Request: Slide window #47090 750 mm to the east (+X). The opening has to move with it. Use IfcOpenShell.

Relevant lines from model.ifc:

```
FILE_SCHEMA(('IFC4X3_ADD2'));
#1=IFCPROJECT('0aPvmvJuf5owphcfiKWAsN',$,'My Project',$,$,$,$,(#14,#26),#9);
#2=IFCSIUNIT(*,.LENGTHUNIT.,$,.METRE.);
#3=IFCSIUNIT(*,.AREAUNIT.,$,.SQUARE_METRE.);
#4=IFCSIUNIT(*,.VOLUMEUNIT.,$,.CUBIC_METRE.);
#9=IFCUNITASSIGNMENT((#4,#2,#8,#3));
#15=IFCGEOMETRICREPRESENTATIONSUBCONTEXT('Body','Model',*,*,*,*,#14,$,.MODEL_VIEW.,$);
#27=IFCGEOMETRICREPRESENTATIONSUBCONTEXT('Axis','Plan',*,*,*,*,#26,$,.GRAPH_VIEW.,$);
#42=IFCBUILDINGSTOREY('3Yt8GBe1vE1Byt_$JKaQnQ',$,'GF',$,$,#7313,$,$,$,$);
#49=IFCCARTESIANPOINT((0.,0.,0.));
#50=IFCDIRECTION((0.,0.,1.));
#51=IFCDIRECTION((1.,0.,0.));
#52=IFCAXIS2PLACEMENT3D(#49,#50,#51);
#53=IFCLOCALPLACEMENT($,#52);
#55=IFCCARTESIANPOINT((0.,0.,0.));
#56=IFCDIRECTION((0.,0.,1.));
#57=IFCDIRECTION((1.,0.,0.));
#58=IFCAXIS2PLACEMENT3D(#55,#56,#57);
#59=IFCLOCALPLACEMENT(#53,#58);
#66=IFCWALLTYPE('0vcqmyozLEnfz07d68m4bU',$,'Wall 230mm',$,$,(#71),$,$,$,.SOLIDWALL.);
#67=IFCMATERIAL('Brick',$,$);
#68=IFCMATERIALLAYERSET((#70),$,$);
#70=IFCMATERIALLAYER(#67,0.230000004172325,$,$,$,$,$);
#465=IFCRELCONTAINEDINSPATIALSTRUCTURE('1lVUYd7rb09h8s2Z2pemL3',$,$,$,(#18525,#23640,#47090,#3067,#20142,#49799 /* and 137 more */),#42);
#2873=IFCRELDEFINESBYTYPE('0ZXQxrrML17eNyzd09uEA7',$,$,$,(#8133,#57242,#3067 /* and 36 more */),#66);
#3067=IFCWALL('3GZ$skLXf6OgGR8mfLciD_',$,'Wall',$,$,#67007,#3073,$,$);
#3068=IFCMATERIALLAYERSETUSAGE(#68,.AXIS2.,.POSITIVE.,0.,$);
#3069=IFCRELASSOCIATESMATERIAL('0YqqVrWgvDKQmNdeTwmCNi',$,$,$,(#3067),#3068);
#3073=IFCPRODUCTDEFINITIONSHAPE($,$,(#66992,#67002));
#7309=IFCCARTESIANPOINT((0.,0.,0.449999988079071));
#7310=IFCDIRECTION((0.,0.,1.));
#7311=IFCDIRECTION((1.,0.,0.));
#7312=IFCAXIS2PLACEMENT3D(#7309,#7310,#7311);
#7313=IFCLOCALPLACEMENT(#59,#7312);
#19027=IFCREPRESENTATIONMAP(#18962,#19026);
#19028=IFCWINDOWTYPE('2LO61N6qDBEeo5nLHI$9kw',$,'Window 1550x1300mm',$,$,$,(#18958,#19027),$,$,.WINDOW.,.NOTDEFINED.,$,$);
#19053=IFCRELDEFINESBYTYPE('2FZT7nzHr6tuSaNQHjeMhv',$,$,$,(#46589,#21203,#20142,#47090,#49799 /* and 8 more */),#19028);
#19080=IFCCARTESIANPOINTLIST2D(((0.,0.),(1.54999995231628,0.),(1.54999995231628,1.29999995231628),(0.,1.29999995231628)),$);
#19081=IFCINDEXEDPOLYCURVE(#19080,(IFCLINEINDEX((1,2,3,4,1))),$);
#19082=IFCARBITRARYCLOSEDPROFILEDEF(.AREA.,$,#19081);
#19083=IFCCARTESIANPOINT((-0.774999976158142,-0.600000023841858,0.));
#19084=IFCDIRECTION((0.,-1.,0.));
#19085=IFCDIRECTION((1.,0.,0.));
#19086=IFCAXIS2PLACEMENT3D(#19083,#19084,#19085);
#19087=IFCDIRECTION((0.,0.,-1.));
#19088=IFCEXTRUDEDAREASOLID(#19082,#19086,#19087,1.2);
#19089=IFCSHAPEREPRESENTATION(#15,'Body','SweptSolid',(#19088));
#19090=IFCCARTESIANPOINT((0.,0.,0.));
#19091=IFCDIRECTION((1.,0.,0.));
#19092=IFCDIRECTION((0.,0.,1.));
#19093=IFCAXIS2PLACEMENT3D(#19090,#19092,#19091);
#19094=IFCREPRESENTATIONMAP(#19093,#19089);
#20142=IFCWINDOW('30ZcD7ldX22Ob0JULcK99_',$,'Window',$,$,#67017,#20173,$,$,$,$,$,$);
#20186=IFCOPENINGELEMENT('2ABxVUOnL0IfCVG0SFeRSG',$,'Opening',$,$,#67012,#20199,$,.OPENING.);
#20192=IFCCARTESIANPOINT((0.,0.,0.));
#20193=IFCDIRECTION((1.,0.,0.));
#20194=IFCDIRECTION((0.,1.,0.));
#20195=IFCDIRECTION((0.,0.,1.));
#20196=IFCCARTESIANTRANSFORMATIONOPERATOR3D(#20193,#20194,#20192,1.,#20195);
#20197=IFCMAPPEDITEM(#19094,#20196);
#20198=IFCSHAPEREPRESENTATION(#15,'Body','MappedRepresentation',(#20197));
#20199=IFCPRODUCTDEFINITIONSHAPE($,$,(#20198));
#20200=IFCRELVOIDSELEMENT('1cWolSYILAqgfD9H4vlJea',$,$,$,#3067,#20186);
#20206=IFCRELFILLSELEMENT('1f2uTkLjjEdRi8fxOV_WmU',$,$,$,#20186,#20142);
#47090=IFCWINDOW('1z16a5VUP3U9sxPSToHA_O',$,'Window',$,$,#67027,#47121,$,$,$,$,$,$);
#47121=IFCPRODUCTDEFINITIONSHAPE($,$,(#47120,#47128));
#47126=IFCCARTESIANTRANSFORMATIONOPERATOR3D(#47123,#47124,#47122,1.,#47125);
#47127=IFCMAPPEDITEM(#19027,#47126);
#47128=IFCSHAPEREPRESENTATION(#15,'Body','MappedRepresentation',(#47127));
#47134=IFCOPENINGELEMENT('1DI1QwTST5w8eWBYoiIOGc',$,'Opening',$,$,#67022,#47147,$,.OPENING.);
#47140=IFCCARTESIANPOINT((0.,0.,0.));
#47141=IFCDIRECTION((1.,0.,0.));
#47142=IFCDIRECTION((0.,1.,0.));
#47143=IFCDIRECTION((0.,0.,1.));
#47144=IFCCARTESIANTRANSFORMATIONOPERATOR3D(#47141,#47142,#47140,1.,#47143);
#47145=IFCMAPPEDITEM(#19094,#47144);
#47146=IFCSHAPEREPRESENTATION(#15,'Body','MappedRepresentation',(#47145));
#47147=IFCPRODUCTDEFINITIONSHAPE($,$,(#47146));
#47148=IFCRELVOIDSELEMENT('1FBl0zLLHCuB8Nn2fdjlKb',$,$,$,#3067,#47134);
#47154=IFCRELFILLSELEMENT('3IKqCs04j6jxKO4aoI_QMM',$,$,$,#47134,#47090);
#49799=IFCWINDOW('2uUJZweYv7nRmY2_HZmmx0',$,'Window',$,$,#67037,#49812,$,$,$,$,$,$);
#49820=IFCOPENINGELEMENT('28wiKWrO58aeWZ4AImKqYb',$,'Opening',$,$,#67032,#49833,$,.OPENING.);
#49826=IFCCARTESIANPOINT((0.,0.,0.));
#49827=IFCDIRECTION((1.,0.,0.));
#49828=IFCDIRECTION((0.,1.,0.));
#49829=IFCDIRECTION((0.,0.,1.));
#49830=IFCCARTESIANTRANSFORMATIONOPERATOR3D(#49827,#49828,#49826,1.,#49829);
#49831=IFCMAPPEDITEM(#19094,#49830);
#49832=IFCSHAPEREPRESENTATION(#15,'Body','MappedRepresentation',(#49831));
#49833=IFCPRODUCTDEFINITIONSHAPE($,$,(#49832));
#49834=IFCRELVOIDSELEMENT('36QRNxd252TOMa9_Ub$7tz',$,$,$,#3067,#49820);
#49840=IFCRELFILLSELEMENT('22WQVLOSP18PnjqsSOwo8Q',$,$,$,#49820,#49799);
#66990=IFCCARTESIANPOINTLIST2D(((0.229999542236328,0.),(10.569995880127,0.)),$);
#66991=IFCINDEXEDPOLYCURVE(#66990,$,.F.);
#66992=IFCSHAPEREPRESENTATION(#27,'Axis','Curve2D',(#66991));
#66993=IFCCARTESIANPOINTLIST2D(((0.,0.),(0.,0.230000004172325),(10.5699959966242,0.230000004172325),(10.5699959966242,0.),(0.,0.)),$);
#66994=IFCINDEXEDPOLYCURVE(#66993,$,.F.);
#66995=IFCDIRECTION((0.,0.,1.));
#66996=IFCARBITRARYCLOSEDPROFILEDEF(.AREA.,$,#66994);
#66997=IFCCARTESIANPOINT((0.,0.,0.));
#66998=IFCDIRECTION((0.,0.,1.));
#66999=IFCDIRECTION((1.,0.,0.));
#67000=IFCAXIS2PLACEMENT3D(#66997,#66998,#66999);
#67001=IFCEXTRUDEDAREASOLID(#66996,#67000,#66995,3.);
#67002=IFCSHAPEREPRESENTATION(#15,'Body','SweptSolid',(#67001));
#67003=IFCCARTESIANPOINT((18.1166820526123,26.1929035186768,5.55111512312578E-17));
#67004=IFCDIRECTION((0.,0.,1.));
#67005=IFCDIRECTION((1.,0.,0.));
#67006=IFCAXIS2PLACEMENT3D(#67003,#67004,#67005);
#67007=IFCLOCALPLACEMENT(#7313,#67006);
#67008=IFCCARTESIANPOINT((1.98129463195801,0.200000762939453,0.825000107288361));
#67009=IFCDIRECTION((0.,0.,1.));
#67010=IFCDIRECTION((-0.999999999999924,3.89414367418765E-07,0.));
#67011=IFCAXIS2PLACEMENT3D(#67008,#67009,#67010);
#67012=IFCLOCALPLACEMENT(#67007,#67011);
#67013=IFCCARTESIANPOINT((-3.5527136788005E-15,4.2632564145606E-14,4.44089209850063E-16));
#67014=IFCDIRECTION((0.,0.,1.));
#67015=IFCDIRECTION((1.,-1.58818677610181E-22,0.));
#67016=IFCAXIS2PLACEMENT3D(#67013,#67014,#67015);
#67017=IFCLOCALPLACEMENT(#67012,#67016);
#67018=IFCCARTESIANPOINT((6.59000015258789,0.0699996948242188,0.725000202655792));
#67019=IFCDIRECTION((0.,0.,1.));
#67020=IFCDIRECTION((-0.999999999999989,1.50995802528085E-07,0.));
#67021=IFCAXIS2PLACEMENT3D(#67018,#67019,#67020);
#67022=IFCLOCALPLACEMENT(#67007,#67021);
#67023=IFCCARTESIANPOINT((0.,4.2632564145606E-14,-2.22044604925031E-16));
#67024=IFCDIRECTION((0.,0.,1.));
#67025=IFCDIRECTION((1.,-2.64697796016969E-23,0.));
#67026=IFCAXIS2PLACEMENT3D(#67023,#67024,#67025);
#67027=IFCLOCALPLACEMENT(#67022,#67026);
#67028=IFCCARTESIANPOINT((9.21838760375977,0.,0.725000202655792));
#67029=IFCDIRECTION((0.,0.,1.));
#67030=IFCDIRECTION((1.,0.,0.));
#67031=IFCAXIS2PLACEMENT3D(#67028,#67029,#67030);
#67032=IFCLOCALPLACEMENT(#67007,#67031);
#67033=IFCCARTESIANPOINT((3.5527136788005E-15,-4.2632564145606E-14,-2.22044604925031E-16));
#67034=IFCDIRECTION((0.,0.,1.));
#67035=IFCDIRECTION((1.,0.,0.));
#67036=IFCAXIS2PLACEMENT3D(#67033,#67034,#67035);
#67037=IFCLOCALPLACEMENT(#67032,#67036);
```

```python
import ifcopenshell
import ifcopenshell.api.geometry
import ifcopenshell.util.placement

model = ifcopenshell.open("model.ifc")

window = model.by_id(47090)
opening = window.FillsVoids[0].RelatingOpeningElement
wall = opening.VoidsElements[0].RelatingBuildingElement

wall_matrix = ifcopenshell.util.placement.get_local_placement(wall.ObjectPlacement)
shift = wall_matrix[:3, 0] * 0.75
before = ifcopenshell.util.placement.get_local_placement(window.ObjectPlacement)[:3, 3].copy()

# The window is placed relative to its opening, so it follows when the opening moves.
matrix = ifcopenshell.util.placement.get_local_placement(opening.ObjectPlacement)
matrix[:3, 3] += shift
ifcopenshell.api.geometry.edit_object_placement(
    model, product=opening, matrix=matrix, is_si=False, should_transform_children=True
)

after = ifcopenshell.util.placement.get_local_placement(window.ObjectPlacement)[:3, 3]
print("window moved by", (after - before).round(3) + 0.0)

model.write("model_edited.ifc")
```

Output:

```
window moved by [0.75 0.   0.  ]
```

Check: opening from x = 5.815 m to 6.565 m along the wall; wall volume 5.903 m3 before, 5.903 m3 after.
